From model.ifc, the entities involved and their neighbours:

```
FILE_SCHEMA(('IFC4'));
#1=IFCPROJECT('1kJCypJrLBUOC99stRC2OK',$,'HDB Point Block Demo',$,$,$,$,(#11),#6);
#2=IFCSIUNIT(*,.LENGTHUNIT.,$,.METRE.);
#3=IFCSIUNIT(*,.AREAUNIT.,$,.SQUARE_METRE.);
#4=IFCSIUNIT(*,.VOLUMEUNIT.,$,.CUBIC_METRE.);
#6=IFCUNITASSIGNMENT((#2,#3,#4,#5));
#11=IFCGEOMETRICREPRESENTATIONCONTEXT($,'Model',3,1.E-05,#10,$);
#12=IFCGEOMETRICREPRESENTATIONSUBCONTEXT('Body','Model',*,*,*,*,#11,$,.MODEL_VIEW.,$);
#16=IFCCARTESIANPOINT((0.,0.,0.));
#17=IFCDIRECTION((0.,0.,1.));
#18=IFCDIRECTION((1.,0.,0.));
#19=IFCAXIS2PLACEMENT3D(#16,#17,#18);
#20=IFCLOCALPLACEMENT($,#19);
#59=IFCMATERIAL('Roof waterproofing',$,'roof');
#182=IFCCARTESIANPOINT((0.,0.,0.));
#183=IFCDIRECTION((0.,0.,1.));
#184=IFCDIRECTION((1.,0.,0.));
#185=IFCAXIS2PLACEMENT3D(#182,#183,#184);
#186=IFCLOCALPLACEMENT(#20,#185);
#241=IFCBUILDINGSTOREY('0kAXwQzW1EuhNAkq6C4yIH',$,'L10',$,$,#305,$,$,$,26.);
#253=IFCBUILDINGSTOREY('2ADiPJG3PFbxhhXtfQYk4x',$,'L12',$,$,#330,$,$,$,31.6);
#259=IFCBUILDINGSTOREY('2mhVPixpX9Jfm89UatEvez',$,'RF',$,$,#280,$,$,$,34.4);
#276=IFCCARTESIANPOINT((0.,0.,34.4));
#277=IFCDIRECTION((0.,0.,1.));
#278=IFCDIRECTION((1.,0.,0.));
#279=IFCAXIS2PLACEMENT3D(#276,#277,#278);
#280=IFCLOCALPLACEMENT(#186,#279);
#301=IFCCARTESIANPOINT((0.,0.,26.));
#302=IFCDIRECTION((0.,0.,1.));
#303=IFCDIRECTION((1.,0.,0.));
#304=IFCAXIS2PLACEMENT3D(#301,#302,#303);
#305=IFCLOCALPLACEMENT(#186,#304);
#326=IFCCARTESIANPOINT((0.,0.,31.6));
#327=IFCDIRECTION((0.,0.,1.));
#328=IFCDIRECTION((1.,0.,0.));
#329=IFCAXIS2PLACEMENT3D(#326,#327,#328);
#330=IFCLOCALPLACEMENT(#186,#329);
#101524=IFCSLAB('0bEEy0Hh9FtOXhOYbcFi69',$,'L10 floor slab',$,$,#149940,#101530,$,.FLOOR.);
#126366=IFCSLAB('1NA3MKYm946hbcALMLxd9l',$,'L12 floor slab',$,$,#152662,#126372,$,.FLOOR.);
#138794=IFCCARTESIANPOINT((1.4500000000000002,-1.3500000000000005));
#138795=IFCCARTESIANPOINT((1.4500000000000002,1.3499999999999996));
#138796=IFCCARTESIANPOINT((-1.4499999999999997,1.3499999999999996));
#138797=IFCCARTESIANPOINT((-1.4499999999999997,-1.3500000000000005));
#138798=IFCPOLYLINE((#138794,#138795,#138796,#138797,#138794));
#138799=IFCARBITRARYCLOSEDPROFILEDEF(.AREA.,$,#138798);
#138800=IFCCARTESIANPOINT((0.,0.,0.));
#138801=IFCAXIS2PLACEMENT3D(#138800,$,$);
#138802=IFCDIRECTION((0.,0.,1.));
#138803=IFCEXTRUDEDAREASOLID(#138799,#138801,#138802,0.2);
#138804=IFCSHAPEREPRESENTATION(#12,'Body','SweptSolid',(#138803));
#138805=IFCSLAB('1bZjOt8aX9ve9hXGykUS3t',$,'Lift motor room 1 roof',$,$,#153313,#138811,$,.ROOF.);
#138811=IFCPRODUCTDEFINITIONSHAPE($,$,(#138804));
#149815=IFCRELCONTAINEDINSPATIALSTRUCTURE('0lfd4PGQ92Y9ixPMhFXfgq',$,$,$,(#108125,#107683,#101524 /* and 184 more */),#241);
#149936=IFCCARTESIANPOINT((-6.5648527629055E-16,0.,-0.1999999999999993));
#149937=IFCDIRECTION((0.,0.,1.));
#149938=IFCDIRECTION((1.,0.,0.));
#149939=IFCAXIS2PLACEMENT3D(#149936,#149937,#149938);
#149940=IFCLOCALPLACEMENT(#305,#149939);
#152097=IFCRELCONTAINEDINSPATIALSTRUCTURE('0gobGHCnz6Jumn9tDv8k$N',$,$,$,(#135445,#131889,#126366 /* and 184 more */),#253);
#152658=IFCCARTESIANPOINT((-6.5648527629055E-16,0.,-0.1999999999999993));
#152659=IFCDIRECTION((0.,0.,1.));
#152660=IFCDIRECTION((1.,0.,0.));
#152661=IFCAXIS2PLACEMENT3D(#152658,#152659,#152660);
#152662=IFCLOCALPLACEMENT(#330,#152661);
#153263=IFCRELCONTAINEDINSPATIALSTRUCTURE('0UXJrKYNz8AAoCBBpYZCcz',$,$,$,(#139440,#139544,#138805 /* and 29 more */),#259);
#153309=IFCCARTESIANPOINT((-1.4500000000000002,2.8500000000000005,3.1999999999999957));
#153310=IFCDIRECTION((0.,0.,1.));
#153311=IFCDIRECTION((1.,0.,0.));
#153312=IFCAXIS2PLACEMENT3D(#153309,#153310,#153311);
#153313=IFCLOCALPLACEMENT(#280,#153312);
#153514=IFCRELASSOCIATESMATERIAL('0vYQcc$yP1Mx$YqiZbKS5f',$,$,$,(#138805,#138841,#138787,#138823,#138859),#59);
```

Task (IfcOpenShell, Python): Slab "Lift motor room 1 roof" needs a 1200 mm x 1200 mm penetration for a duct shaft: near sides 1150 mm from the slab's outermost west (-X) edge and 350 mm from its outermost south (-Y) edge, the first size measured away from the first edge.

```python
import numpy as np
import ifcopenshell
import ifcopenshell.api.feature
import ifcopenshell.api.geometry
import ifcopenshell.api.root
import ifcopenshell.geom
import ifcopenshell.util.placement
import ifcopenshell.util.representation
import ifcopenshell.util.shape
import ifcopenshell.util.unit

model = ifcopenshell.open("model.ifc")
unit_scale = ifcopenshell.util.unit.calculate_unit_scale(model)
settings = ifcopenshell.geom.settings()


def volume(element):
    """Net volume in cubic metres, openings subtracted."""
    shape = ifcopenshell.geom.create_shape(settings, element)
    return ifcopenshell.util.shape.get_volume(shape.geometry)


slab = model.by_guid("1bZjOt8aX9ve9hXGykUS3t")
before = volume(slab)

# Extent in the slab's own axes, in metres. The edges named are its -X and -Y sides.
slab_shape = ifcopenshell.geom.create_shape(settings, slab)
vertices = ifcopenshell.util.shape.get_vertices(slab_shape.geometry)
x_min, y_min, bottom = vertices.min(axis=0)
top = vertices[:, 2].max()

opening = ifcopenshell.api.root.create_entity(model, ifc_class="IfcOpeningElement", name="Duct shaft opening", predefined_type="OPENING")
context = ifcopenshell.util.representation.get_context(model, "Model", "Body", "MODEL_VIEW")
width, depth = 1.2, 1.2
outline = [(0.0, 0.0), (width, 0.0), (width, depth), (0.0, depth), (0.0, 0.0)]
# Overshoot both faces by 50 mm so the cut is clean.
shape = ifcopenshell.api.geometry.add_slab_representation(
    model, context=context, depth=top - bottom + 0.1, polyline=outline
)
ifcopenshell.api.geometry.assign_representation(model, product=opening, representation=shape)

matrix = ifcopenshell.util.placement.get_local_placement(slab.ObjectPlacement)
matrix[:, 3] = matrix @ np.append(np.array([x_min + 1.15, y_min + 0.35, bottom - 0.05]) / unit_scale, 1.0)
ifcopenshell.api.geometry.edit_object_placement(model, product=opening, matrix=matrix, is_si=False)
ifcopenshell.api.feature.add_feature(model, feature=opening, element=slab)

after = volume(slab)

print(f"slab volume {before:.3f} -> {after:.3f} m3")

model.write("model_edited.ifc")
```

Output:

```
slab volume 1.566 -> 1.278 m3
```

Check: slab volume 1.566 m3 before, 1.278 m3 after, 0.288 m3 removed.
